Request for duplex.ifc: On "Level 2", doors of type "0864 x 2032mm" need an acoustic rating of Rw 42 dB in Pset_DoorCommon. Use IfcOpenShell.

First a look at what the model holds.

```python
import ifcopenshell
import ifcopenshell.util.element

model = ifcopenshell.open("duplex.ifc")
print(model.schema)
storey = next(s for s in model.by_type("IfcBuildingStorey") if s.Name == "Level 2")
doors = [e for e in ifcopenshell.util.element.get_decomposition(storey) if e.is_a("IfcDoor")]
seen = {}
for e in doors:
    element_type = ifcopenshell.util.element.get_type(e)
    key = (element_type.Name if element_type != e and element_type else None, ifcopenshell.util.element.get_pset(e, "Pset_DoorCommon", "AcousticRating"))
    seen[key] = seen.get(key, 0) + 1
for (name, value), count in sorted(seen.items(), key=str):
    print(count, "x", name, "|", value)
```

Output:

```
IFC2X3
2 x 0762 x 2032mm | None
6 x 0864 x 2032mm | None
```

```python
import ifcopenshell
import ifcopenshell.api.pset
import ifcopenshell.util.element

model = ifcopenshell.open("duplex.ifc")

storey = next(s for s in model.by_type("IfcBuildingStorey") if s.Name == "Level 2")
doors = [e for e in ifcopenshell.util.element.get_decomposition(storey) if e.is_a("IfcDoor")]

count = 0
for e in doors:
    element_type = ifcopenshell.util.element.get_type(e)
    if element_type in (None, e) or element_type.Name != "0864 x 2032mm":
        continue
    # add_pset returns the element's existing set when there is one.
    pset = ifcopenshell.api.pset.add_pset(model, product=e, name="Pset_DoorCommon")
    ifcopenshell.api.pset.edit_pset(model, pset=pset, properties={"AcousticRating": "Rw 42 dB"})
    count += 1

print(count, "doors updated")

model.write("duplex_rev.ifc")
```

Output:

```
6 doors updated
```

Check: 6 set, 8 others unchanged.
